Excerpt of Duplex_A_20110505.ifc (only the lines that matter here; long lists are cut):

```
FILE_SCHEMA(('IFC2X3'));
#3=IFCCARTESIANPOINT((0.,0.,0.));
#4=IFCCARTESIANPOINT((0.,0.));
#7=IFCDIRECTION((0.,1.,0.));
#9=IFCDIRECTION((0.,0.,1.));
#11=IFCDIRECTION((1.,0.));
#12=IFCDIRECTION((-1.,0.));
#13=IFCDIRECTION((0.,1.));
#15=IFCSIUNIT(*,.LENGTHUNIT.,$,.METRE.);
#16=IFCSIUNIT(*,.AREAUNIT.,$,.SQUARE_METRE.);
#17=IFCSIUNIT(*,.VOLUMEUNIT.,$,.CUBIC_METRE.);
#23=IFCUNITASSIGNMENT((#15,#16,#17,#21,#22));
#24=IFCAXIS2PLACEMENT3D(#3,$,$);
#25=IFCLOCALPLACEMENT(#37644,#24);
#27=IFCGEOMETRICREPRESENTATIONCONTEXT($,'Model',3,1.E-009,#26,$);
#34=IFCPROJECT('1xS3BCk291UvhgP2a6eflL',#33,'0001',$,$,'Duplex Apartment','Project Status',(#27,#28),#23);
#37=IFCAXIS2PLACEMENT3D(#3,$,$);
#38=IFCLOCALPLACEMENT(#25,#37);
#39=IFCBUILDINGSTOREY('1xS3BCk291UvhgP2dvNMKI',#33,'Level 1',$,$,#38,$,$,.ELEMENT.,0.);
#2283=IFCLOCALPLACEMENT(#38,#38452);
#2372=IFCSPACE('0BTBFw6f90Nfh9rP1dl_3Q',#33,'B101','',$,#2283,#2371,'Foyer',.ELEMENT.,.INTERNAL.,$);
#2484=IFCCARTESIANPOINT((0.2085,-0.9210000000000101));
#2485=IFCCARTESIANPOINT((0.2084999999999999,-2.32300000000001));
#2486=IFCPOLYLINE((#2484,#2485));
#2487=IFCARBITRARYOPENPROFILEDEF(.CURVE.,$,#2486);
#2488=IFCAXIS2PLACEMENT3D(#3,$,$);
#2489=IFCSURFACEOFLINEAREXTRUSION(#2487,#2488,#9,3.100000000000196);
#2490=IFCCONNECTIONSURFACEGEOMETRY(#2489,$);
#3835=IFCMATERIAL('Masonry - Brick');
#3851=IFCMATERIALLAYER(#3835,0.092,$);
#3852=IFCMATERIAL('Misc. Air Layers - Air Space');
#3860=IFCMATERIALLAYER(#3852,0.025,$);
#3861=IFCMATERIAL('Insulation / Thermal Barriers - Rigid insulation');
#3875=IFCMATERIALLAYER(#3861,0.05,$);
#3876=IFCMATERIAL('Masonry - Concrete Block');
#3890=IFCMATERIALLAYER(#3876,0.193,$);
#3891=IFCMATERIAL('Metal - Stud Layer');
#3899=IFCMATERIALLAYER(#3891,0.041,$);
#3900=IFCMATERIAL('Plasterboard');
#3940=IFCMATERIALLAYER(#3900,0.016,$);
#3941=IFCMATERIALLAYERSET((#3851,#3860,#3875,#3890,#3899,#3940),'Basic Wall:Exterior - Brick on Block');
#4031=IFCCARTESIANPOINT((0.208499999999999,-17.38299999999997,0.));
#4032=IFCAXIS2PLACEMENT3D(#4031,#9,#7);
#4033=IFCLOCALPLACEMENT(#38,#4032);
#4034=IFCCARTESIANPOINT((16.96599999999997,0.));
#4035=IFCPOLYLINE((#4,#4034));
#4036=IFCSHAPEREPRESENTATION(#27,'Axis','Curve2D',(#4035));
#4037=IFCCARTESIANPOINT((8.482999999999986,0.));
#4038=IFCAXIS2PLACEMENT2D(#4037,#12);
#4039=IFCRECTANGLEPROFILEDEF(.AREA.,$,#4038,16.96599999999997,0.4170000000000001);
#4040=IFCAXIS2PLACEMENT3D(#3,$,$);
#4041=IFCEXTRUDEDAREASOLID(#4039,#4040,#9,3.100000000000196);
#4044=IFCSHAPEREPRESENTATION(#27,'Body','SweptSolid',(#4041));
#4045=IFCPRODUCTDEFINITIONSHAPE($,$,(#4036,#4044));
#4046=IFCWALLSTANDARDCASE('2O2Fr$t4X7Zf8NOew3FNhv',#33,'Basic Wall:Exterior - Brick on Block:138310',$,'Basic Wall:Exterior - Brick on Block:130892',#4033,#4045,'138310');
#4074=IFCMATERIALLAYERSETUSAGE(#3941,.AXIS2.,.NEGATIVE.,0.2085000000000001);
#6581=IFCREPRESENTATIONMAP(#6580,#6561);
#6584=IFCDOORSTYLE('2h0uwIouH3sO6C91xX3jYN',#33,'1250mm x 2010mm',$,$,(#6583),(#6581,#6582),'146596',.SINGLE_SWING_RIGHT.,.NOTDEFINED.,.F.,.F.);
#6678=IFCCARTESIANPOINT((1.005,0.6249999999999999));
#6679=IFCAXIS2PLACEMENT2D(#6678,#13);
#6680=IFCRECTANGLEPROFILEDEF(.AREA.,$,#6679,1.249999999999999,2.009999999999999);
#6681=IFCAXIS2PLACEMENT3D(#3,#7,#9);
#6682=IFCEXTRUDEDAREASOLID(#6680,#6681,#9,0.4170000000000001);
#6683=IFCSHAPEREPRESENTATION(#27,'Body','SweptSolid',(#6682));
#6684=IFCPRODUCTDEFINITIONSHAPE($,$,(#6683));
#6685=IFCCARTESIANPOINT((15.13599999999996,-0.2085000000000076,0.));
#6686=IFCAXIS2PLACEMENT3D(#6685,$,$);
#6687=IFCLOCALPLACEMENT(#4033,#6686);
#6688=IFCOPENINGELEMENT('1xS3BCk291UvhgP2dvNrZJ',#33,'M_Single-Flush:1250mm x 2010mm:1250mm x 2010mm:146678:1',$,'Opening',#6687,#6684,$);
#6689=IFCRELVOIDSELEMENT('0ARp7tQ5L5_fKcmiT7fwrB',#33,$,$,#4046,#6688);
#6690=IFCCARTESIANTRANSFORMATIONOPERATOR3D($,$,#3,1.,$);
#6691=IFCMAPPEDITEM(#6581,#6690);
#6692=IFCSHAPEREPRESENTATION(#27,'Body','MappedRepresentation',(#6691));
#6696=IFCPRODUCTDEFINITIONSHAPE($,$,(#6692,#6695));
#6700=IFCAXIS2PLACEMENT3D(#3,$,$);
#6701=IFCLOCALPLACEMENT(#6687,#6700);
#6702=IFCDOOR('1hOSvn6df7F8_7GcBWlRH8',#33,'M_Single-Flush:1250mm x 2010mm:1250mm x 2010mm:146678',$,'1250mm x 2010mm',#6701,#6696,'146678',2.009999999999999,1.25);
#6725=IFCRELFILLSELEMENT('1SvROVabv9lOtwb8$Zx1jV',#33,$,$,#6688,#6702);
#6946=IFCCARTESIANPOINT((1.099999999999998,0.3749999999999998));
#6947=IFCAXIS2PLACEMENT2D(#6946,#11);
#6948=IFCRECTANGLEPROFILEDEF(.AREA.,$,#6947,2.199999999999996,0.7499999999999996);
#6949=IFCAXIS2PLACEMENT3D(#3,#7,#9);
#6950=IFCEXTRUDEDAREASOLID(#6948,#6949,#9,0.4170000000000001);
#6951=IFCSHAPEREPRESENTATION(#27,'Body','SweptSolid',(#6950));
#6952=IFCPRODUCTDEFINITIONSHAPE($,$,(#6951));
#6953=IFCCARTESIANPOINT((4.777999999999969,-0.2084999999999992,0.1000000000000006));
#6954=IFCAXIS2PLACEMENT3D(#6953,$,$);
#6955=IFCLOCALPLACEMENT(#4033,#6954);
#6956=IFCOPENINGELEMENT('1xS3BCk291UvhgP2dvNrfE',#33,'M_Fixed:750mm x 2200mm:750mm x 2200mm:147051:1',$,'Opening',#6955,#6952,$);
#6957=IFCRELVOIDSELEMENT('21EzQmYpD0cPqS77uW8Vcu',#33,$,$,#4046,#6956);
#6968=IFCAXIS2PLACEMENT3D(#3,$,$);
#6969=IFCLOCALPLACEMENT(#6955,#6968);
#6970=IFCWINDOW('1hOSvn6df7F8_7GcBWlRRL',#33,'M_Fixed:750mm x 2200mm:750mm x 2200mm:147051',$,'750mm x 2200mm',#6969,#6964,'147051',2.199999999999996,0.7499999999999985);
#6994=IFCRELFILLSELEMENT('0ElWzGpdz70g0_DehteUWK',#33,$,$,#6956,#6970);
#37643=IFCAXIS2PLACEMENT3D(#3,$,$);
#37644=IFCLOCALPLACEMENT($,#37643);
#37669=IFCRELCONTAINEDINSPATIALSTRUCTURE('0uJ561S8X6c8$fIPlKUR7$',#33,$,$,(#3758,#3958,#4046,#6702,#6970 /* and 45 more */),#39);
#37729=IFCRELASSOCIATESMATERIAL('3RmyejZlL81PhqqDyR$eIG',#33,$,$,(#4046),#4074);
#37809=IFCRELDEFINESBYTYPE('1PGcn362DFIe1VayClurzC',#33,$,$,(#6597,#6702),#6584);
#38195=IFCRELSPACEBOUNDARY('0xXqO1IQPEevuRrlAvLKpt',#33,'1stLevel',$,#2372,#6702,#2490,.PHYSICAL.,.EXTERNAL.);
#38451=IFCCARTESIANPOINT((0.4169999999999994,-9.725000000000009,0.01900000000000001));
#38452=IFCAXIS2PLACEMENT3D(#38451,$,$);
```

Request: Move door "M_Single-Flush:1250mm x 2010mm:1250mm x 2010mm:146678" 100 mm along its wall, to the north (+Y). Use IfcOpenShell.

```python
import numpy as np
import ifcopenshell
import ifcopenshell.api.geometry
import ifcopenshell.util.placement
import ifcopenshell.util.unit

model = ifcopenshell.open("Duplex_A_20110505.ifc")
unit_scale = ifcopenshell.util.unit.calculate_unit_scale(model)

door = model.by_guid("1hOSvn6df7F8_7GcBWlRH8")
opening = door.FillsVoids[0].RelatingOpeningElement
wall = opening.VoidsElements[0].RelatingBuildingElement

wall_matrix = ifcopenshell.util.placement.get_local_placement(wall.ObjectPlacement)
shift = wall_matrix[:3, 0] * 0.1 / unit_scale
before = ifcopenshell.util.placement.get_local_placement(door.ObjectPlacement)[:3, 3].copy()

# The door is placed relative to its opening, so it follows when the opening moves.
matrix = ifcopenshell.util.placement.get_local_placement(opening.ObjectPlacement)
matrix[:3, 3] += shift
ifcopenshell.api.geometry.edit_object_placement(
    model, product=opening, matrix=matrix, is_si=False, should_transform_children=True
)

# Space boundary surfaces are stored in each space's coordinates; move them too.
for rel in door.ProvidesBoundaries:
    if not rel.ConnectionGeometry:
        continue
    surface = rel.ConnectionGeometry.SurfaceOnRelatingElement
    space_matrix = ifcopenshell.util.placement.get_local_placement(rel.RelatingSpace.ObjectPlacement)
    point = np.array(surface.Position.Location.Coordinates) + space_matrix[:3, :3].T @ shift
    surface.Position = model.createIfcAxis2Placement3D(
        model.createIfcCartesianPoint(point.tolist()), surface.Position.Axis, surface.Position.RefDirection
    )

after = ifcopenshell.util.placement.get_local_placement(door.ObjectPlacement)[:3, 3]
print("door moved by", (after - before).round(3) + 0.0)

model.write("Duplex_A_20110505-out.ifc")
```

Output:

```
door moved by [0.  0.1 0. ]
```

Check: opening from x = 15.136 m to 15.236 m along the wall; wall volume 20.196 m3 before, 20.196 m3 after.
